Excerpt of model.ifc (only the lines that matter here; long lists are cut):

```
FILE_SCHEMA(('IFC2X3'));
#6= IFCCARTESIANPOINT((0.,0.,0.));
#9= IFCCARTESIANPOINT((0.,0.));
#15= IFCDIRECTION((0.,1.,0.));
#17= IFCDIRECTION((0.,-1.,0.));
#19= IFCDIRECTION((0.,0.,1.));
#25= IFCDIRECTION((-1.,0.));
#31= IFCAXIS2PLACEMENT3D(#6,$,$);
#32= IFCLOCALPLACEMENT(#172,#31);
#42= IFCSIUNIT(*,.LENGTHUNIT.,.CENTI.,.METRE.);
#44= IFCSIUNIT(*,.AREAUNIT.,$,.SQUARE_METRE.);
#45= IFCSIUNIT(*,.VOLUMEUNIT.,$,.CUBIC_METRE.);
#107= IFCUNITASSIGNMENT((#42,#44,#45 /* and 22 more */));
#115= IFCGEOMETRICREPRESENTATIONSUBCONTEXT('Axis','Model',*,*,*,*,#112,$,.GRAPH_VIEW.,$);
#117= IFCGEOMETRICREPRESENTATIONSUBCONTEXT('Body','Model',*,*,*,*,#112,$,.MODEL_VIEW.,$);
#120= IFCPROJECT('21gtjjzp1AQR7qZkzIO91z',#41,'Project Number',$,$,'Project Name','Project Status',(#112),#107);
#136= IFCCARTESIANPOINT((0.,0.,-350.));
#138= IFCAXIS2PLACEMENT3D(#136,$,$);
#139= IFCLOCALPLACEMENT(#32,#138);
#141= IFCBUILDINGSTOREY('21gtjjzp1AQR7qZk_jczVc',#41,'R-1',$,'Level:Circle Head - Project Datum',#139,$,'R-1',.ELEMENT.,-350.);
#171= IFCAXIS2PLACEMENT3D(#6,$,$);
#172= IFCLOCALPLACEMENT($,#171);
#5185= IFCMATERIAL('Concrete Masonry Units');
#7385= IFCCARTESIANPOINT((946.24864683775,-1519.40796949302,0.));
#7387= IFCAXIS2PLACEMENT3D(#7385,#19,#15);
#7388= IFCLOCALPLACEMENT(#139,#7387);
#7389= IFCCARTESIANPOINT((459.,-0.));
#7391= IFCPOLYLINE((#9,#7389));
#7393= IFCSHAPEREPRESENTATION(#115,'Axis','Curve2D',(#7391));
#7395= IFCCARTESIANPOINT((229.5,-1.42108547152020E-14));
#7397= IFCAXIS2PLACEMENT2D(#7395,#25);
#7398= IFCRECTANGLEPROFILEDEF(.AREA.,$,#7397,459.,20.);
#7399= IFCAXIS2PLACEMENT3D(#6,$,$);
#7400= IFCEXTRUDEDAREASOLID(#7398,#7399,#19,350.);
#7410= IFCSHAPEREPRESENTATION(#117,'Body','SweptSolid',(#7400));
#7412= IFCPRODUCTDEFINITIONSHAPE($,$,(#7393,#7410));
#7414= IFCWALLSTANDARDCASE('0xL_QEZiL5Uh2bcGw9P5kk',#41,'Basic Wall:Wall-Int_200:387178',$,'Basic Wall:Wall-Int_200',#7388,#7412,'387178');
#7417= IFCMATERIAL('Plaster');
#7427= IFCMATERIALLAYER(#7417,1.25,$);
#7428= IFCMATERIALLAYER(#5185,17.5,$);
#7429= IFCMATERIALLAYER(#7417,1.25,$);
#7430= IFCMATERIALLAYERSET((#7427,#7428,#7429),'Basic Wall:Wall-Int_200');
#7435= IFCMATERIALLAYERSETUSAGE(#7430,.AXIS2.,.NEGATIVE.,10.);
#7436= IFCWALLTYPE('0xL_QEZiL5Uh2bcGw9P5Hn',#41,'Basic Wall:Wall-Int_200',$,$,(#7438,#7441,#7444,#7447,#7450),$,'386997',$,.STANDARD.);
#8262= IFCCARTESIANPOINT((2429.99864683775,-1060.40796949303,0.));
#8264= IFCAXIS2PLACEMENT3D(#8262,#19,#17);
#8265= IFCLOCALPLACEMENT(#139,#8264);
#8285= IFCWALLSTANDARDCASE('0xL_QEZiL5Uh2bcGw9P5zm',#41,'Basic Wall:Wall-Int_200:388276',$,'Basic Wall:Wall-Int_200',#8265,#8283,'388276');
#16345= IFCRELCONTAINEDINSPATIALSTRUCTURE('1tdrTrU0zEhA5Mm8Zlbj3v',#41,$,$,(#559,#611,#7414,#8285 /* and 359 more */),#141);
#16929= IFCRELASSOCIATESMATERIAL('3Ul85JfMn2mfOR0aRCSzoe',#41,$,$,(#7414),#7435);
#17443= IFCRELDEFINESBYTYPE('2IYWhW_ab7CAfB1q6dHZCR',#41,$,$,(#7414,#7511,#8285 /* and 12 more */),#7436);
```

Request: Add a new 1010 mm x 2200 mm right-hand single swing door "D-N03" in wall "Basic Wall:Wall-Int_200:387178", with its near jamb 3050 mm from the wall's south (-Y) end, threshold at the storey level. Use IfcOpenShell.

```python
import numpy as np
import ifcopenshell
import ifcopenshell.api.feature
import ifcopenshell.api.geometry
import ifcopenshell.api.root
import ifcopenshell.api.spatial
import ifcopenshell.api.type
import ifcopenshell.geom
import ifcopenshell.util.element
import ifcopenshell.util.placement
import ifcopenshell.util.representation
import ifcopenshell.util.shape
import ifcopenshell.util.unit

model = ifcopenshell.open("model.ifc")
unit_scale = ifcopenshell.util.unit.calculate_unit_scale(model)
settings = ifcopenshell.geom.settings()


def volume(element):
    """Net volume in cubic metres, openings subtracted."""
    shape = ifcopenshell.geom.create_shape(settings, element)
    return ifcopenshell.util.shape.get_volume(shape.geometry)


wall = model.by_guid("0xL_QEZiL5Uh2bcGw9P5kk")
storey = ifcopenshell.util.element.get_container(wall, ifc_class="IfcBuildingStorey")
context = ifcopenshell.util.representation.get_context(model, "Model", "Body", "MODEL_VIEW")
before = volume(wall)

width, height, from_end, sill = 1.01, 2.2, 3.05, 0.0  # metres

# The wall runs along its own X axis, and the end named is its -X end.
wall_shape = ifcopenshell.geom.create_shape(settings, wall)
x, y, z = ifcopenshell.util.shape.get_vertices(wall_shape.geometry).T
start = x.min() + from_end
face, thickness = float(y.min()), float(y.max() - y.min())
wall_matrix = ifcopenshell.util.placement.get_local_placement(wall.ObjectPlacement)
level = ifcopenshell.util.placement.get_local_placement(storey.ObjectPlacement)[2, 3]


def in_wall(x, y):
    """Placement at x, y metres in the wall's axes, at sill height."""
    matrix = wall_matrix.copy()
    matrix[:, 3] = wall_matrix @ np.array([x / unit_scale, y / unit_scale, 0.0, 1.0])
    matrix[2, 3] = level + sill / unit_scale
    return matrix


# Opening: a box that overshoots both wall faces by 50 mm.
opening = ifcopenshell.api.root.create_entity(model, ifc_class="IfcOpeningElement")
box = ifcopenshell.api.geometry.add_wall_representation(
    model, context=context, length=width, height=height, thickness=thickness + 0.1
)
ifcopenshell.api.geometry.assign_representation(model, product=opening, representation=box)
ifcopenshell.api.geometry.edit_object_placement(model, product=opening, matrix=in_wall(start, face - 0.05), is_si=False)
ifcopenshell.api.feature.add_feature(model, feature=opening, element=wall)

door = ifcopenshell.api.root.create_entity(model, ifc_class="IfcDoor", name="D-N03")
door.OverallWidth, door.OverallHeight = width / unit_scale, height / unit_scale
body = ifcopenshell.api.geometry.add_door_representation(
    model,
    context=context,
    overall_width=door.OverallWidth,
    overall_height=door.OverallHeight,
    operation_type="SINGLE_SWING_RIGHT",
    lining_properties={"LiningDepth": thickness / unit_scale, "ThresholdDepth": thickness / unit_scale},
)
ifcopenshell.api.geometry.assign_representation(model, product=door, representation=body)
ifcopenshell.api.spatial.assign_container(model, products=[door], relating_structure=storey)
fills = ifcopenshell.api.feature.add_filling(model, opening=opening, element=door)
fills.OwnerHistory = door.OwnerHistory  # required in IFC2X3

# IFC2X3 keeps the operation on the door style.
style = ifcopenshell.api.root.create_entity(model, ifc_class="IfcDoorStyle", name="D-N03")
style.OperationType, style.ConstructionType = "SINGLE_SWING_RIGHT", "NOTDEFINED"
style.ParameterTakesPrecedence = style.Sizeable = False
ifcopenshell.api.type.assign_type(model, related_objects=[door], relating_type=style)

# The lining spans the wall, so the door starts at the wall face.
ifcopenshell.api.geometry.edit_object_placement(model, product=door, matrix=in_wall(start, face), is_si=False)

after = volume(wall)

print(f"wall volume {before:.3f} -> {after:.3f} m3")

model.write("model-out.ifc")
```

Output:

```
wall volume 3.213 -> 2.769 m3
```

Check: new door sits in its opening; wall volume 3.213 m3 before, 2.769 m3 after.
